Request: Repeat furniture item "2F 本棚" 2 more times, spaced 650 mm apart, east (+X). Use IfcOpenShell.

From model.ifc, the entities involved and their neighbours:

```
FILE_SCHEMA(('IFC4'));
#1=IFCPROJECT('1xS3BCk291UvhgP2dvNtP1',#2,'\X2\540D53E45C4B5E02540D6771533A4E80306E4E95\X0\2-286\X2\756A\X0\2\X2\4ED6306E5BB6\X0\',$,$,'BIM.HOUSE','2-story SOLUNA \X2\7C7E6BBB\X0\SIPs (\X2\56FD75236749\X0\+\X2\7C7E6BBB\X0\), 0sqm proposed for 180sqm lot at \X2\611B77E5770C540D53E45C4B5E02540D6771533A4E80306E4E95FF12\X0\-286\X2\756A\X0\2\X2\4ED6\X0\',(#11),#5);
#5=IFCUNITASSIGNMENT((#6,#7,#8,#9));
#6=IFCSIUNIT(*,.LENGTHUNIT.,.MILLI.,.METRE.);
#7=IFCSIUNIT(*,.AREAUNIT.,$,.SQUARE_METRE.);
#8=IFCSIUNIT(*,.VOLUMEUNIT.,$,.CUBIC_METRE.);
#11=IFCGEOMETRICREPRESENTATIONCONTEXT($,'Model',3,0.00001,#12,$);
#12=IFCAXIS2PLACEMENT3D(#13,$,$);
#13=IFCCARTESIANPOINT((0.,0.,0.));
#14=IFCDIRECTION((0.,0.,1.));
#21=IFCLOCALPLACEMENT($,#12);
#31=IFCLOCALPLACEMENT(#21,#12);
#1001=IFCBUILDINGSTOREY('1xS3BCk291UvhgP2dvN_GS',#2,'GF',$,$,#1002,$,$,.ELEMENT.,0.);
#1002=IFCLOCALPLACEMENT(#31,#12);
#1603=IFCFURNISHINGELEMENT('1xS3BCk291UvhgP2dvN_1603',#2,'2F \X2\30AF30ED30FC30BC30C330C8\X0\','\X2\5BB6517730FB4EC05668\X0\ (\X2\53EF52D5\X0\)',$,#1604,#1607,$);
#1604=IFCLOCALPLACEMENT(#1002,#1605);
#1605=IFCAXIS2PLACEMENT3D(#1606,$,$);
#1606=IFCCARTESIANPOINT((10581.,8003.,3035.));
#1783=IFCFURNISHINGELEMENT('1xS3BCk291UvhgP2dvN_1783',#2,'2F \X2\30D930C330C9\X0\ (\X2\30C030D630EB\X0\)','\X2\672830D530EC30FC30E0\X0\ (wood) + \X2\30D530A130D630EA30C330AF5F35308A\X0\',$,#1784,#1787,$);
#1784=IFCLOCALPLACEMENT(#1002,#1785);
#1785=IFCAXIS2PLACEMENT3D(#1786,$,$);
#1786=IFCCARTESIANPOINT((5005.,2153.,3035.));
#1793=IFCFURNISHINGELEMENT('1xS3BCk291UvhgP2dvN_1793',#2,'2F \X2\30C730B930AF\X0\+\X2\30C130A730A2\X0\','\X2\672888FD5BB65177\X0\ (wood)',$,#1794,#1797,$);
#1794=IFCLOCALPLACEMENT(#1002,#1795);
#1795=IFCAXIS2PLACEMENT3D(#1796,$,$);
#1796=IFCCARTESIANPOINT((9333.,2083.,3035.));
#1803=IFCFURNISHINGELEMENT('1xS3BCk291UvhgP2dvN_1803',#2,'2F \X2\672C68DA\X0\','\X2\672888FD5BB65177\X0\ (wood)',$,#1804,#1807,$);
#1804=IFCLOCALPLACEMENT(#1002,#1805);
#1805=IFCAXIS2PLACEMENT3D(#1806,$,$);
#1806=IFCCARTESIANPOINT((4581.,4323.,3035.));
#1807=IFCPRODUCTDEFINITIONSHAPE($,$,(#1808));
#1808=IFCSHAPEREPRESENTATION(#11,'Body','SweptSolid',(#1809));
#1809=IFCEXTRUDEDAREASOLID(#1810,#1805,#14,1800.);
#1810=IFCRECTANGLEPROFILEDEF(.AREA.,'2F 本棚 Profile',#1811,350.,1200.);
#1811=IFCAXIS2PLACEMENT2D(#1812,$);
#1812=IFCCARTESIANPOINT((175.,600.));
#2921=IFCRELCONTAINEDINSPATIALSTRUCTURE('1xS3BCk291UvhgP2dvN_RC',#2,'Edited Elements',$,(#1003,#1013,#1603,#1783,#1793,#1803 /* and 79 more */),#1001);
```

```python
import numpy as np
import ifcopenshell
import ifcopenshell.api.geometry
import ifcopenshell.api.root
import ifcopenshell.util.element
import ifcopenshell.util.placement

model = ifcopenshell.open("model.ifc")


def reuse_history(source, copy):
    """copy_class also copies each property set's owner history, people and application; keep the originals."""
    for rel in copy.IsDefinedBy:
        if rel.is_a("IfcRelDefinesByProperties") and (history := rel.RelatingPropertyDefinition.OwnerHistory):
            rel.RelatingPropertyDefinition.OwnerHistory = source.OwnerHistory
            ifcopenshell.util.element.remove_deep2(model, history)


source = model.by_id(1803)
base = ifcopenshell.util.placement.get_local_placement(source.ObjectPlacement)
step = np.array([1.0, 0.0, 0.0]) * 650.0

for i in range(1, 3):
    copy = ifcopenshell.api.root.copy_class(model, product=source)
    copy.Representation = ifcopenshell.util.element.copy_deep(
        model, source.Representation, exclude=["IfcGeometricRepresentationContext", "IfcRepresentationMap"]
    )
    reuse_history(source, copy)
    matrix = base.copy()
    matrix[:3, 3] += i * step
    print("added at", matrix[:3, 3].round(3) + 0.0)
    ifcopenshell.api.geometry.edit_object_placement(model, product=copy, matrix=matrix, is_si=False)

model.write("model_edited.ifc")
```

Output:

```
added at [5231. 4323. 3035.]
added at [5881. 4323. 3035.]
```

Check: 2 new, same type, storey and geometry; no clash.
